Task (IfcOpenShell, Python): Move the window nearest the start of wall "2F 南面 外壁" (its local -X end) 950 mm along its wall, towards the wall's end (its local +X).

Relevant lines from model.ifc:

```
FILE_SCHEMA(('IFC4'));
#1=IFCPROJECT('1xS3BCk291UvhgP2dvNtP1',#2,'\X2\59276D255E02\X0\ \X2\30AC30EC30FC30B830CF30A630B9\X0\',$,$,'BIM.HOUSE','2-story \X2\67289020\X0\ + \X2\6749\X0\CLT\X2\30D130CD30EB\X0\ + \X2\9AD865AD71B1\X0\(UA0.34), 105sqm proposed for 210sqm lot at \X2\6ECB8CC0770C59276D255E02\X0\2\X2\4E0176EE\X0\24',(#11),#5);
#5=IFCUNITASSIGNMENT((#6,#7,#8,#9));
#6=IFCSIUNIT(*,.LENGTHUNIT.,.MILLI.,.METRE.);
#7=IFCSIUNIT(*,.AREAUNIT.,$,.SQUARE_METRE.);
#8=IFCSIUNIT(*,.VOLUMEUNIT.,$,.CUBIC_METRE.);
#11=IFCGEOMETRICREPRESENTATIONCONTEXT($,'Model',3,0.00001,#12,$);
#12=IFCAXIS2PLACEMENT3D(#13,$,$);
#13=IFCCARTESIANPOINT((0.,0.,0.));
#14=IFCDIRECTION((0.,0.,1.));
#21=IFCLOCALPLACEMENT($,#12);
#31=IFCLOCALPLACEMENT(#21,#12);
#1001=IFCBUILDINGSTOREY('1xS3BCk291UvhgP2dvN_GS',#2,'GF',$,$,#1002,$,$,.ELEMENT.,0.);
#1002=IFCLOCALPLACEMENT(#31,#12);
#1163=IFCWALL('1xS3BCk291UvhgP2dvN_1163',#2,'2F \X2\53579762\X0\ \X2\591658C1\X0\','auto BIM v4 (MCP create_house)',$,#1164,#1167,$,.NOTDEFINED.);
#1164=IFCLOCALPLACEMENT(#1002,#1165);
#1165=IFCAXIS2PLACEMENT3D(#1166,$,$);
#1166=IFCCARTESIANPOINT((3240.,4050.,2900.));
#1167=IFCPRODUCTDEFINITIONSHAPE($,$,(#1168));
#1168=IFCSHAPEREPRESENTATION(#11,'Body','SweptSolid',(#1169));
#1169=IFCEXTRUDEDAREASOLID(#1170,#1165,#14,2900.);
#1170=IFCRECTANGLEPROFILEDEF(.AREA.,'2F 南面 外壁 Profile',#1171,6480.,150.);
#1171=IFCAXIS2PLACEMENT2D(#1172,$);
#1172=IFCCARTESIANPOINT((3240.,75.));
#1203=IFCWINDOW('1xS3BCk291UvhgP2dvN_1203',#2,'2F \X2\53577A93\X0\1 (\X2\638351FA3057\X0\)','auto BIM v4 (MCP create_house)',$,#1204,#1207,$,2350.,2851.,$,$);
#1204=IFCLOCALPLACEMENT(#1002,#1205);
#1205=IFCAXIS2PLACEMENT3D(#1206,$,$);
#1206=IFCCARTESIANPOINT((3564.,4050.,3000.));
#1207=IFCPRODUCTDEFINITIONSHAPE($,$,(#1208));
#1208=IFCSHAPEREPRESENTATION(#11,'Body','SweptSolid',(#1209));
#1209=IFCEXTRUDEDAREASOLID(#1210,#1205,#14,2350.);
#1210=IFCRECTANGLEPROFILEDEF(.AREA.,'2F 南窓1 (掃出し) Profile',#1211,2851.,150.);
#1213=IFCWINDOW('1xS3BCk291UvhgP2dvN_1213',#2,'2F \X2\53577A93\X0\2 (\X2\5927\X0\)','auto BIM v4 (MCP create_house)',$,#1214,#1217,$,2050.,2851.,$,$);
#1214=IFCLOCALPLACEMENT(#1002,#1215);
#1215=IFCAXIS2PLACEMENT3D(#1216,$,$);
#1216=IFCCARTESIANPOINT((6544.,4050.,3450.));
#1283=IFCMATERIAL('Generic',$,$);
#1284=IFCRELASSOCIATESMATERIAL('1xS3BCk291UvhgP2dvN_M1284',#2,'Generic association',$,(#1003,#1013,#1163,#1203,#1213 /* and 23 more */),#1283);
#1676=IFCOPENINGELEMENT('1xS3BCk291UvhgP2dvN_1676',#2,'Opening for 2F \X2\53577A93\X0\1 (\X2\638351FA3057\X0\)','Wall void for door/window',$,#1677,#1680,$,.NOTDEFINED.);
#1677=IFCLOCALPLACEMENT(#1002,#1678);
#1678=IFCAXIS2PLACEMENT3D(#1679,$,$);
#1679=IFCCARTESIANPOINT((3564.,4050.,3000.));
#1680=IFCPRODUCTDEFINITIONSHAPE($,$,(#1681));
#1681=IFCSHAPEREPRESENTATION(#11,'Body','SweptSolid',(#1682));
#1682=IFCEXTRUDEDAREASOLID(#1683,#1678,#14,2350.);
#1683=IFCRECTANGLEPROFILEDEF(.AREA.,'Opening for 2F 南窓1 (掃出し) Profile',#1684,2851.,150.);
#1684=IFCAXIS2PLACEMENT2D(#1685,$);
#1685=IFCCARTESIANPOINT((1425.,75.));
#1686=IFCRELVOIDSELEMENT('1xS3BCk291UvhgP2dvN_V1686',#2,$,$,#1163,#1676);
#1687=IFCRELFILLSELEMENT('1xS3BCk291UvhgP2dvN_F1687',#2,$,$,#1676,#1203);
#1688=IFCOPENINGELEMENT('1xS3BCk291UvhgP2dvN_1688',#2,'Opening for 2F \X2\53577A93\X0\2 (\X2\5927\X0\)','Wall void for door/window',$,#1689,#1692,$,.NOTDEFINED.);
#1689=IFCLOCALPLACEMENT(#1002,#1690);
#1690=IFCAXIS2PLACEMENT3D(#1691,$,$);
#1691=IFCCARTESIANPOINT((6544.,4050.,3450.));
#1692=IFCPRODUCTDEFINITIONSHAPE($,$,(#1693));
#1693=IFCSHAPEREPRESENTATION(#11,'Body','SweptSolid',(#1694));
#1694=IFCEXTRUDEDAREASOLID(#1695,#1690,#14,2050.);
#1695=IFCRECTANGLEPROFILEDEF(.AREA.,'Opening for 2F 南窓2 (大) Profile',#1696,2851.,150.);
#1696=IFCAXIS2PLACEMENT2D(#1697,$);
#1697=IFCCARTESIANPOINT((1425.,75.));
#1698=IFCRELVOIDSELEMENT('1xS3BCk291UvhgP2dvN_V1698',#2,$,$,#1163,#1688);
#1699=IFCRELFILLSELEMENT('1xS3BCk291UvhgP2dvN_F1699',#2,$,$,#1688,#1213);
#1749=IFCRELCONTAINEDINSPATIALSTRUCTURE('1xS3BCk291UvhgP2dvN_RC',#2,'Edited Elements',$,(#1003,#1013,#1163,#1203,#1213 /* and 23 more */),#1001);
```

```python
import ifcopenshell
import ifcopenshell.api.geometry
import ifcopenshell.util.placement
import ifcopenshell.util.unit

model = ifcopenshell.open("model.ifc")
unit_scale = ifcopenshell.util.unit.calculate_unit_scale(model)

window = model.by_guid("1xS3BCk291UvhgP2dvN_1203")
opening = window.FillsVoids[0].RelatingOpeningElement
wall = opening.VoidsElements[0].RelatingBuildingElement

wall_matrix = ifcopenshell.util.placement.get_local_placement(wall.ObjectPlacement)
shift = wall_matrix[:3, 0] * 0.95 / unit_scale
before = ifcopenshell.util.placement.get_local_placement(window.ObjectPlacement)[:3, 3].copy()

# The window is not placed relative to its opening, so move both.
for product in (opening, window):
    matrix = ifcopenshell.util.placement.get_local_placement(product.ObjectPlacement)
    matrix[:3, 3] += shift
    ifcopenshell.api.geometry.edit_object_placement(model, product=product, matrix=matrix, is_si=False)

after = ifcopenshell.util.placement.get_local_placement(window.ObjectPlacement)[:3, 3]
print("window moved by", (after - before).round(3) + 0.0)

model.write("model_updated.ifc")
```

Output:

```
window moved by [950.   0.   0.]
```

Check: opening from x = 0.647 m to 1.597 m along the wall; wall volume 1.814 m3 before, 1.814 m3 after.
